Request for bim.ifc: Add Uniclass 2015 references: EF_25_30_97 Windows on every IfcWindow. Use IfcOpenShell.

First a look at what the model holds.

```python
import ifcopenshell

model = ifcopenshell.open("bim.ifc")
print(model.schema)
print("classifications:", [c.Name for c in model.by_type("IfcClassification")])
for ifc_class in ("IfcDoor", "IfcRoof", "IfcStair", "IfcWall", "IfcWindow"):
    print(ifc_class, len(model.by_type(ifc_class)))
```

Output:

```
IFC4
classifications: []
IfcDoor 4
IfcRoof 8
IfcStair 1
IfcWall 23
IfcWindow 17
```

```python
import ifcopenshell
import ifcopenshell.api.classification

model = ifcopenshell.open("bim.ifc")

system = ifcopenshell.api.classification.add_classification(model, classification="Uniclass 2015")

codes = {
    "IfcWindow": ("EF_25_30_97", "Windows"),
}
for ifc_class, (code, name) in codes.items():
    products = model.by_type(ifc_class)
    ifcopenshell.api.classification.add_reference(
        model, products=products, classification=system, identification=code, name=name
    )
    print(code, len(products))

model.write("bim_v2.ifc")
```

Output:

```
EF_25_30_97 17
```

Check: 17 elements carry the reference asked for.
